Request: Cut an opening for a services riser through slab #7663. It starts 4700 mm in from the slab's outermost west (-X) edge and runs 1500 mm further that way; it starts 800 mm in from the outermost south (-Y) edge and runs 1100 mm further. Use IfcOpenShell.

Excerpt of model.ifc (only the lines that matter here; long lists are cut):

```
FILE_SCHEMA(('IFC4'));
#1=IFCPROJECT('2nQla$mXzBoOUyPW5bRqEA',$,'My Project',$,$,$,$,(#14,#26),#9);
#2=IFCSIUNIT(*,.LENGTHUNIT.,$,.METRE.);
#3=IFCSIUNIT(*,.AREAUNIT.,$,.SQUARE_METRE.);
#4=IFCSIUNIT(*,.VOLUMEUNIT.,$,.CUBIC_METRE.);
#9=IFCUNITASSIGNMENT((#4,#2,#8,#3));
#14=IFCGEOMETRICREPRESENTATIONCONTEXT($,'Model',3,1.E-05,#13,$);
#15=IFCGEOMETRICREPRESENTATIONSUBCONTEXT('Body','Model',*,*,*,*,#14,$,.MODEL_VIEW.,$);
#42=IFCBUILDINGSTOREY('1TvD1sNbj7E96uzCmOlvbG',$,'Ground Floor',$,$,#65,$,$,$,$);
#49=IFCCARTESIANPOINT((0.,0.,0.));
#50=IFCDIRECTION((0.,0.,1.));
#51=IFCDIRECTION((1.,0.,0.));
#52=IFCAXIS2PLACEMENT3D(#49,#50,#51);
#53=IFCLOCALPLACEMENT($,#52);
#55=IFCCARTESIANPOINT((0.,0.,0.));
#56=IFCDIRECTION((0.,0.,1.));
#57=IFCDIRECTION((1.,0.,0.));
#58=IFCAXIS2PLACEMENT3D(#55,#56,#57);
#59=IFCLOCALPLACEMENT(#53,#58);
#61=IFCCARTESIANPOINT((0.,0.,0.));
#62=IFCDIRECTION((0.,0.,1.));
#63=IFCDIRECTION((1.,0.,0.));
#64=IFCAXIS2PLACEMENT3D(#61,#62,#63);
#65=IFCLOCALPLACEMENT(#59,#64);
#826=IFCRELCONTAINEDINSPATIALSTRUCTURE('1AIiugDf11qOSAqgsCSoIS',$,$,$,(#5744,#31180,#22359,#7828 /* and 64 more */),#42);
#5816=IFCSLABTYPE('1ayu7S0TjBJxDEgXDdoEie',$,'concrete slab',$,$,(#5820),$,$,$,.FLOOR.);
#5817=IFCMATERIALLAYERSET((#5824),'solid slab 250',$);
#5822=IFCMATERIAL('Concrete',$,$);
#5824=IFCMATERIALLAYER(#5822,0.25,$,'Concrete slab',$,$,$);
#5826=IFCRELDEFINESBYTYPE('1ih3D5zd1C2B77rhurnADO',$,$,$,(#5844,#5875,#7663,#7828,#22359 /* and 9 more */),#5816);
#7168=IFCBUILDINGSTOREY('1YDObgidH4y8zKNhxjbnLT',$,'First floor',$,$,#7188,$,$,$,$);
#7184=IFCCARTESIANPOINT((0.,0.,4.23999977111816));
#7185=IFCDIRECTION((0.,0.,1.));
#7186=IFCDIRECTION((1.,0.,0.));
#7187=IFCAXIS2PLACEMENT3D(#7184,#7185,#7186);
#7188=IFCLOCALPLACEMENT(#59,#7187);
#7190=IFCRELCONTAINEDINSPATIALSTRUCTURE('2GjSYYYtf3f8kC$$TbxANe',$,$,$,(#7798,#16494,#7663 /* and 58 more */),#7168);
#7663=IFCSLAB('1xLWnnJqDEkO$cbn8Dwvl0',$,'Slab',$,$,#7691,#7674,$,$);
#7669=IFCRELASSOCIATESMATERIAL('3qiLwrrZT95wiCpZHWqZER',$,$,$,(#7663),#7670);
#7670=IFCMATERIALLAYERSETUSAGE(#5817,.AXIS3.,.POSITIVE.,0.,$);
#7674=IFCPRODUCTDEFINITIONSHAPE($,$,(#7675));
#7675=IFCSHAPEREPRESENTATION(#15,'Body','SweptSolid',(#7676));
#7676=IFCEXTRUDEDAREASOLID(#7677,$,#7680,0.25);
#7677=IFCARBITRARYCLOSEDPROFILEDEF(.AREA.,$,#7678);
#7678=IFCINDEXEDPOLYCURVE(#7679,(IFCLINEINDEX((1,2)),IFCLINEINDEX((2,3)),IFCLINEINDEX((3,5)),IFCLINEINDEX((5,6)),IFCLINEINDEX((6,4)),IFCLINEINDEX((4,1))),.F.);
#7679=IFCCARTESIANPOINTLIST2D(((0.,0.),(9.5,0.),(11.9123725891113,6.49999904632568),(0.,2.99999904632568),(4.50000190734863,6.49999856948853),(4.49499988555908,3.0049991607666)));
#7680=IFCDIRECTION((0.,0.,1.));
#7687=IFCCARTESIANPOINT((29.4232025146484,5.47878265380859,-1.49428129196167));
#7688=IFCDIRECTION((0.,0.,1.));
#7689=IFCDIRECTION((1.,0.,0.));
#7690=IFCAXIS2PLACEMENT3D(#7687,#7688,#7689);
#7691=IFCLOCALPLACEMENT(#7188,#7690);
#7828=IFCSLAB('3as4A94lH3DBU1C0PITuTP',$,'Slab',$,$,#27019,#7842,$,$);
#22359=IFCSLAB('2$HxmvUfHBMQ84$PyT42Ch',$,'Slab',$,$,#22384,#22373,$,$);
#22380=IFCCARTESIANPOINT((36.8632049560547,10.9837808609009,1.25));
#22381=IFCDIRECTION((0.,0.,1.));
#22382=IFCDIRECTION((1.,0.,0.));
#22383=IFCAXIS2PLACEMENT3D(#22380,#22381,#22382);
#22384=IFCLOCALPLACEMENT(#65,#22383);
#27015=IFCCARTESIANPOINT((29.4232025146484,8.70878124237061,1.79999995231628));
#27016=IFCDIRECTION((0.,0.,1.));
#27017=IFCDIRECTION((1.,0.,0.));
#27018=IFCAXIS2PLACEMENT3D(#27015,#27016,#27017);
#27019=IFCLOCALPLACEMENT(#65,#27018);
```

```python
import numpy as np
import ifcopenshell
import ifcopenshell.api.feature
import ifcopenshell.api.geometry
import ifcopenshell.api.root
import ifcopenshell.geom
import ifcopenshell.util.placement
import ifcopenshell.util.representation
import ifcopenshell.util.shape
import ifcopenshell.util.unit

model = ifcopenshell.open("model.ifc")
unit_scale = ifcopenshell.util.unit.calculate_unit_scale(model)
settings = ifcopenshell.geom.settings()


def volume(element):
    """Net volume in cubic metres, openings subtracted."""
    shape = ifcopenshell.geom.create_shape(settings, element)
    return ifcopenshell.util.shape.get_volume(shape.geometry)


slab = model.by_guid("1xLWnnJqDEkO$cbn8Dwvl0")
before = volume(slab)

# Extent in the slab's own axes, in metres. The edges named are its -X and -Y sides.
slab_shape = ifcopenshell.geom.create_shape(settings, slab)
vertices = ifcopenshell.util.shape.get_vertices(slab_shape.geometry)
x_min, y_min, bottom = vertices.min(axis=0)
top = vertices[:, 2].max()

opening = ifcopenshell.api.root.create_entity(model, ifc_class="IfcOpeningElement", name="Services riser opening", predefined_type="OPENING")
context = ifcopenshell.util.representation.get_context(model, "Model", "Body", "MODEL_VIEW")
width, depth = 1.5, 1.1
outline = [(0.0, 0.0), (width, 0.0), (width, depth), (0.0, depth), (0.0, 0.0)]
# Overshoot both faces by 50 mm so the cut is clean.
shape = ifcopenshell.api.geometry.add_slab_representation(
    model, context=context, depth=top - bottom + 0.1, polyline=outline
)
ifcopenshell.api.geometry.assign_representation(model, product=opening, representation=shape)

matrix = ifcopenshell.util.placement.get_local_placement(slab.ObjectPlacement)
matrix[:, 3] = matrix @ np.append(np.array([x_min + 4.7, y_min + 0.8, bottom - 0.05]) / unit_scale, 1.0)
ifcopenshell.api.geometry.edit_object_placement(model, product=opening, matrix=matrix, is_si=False)
ifcopenshell.api.feature.add_feature(model, feature=opening, element=slab)

after = volume(slab)

print(f"slab volume {before:.3f} -> {after:.3f} m3")

model.write("model_edited.ifc")
```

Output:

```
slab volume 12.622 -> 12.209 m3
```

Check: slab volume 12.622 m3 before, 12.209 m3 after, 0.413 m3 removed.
